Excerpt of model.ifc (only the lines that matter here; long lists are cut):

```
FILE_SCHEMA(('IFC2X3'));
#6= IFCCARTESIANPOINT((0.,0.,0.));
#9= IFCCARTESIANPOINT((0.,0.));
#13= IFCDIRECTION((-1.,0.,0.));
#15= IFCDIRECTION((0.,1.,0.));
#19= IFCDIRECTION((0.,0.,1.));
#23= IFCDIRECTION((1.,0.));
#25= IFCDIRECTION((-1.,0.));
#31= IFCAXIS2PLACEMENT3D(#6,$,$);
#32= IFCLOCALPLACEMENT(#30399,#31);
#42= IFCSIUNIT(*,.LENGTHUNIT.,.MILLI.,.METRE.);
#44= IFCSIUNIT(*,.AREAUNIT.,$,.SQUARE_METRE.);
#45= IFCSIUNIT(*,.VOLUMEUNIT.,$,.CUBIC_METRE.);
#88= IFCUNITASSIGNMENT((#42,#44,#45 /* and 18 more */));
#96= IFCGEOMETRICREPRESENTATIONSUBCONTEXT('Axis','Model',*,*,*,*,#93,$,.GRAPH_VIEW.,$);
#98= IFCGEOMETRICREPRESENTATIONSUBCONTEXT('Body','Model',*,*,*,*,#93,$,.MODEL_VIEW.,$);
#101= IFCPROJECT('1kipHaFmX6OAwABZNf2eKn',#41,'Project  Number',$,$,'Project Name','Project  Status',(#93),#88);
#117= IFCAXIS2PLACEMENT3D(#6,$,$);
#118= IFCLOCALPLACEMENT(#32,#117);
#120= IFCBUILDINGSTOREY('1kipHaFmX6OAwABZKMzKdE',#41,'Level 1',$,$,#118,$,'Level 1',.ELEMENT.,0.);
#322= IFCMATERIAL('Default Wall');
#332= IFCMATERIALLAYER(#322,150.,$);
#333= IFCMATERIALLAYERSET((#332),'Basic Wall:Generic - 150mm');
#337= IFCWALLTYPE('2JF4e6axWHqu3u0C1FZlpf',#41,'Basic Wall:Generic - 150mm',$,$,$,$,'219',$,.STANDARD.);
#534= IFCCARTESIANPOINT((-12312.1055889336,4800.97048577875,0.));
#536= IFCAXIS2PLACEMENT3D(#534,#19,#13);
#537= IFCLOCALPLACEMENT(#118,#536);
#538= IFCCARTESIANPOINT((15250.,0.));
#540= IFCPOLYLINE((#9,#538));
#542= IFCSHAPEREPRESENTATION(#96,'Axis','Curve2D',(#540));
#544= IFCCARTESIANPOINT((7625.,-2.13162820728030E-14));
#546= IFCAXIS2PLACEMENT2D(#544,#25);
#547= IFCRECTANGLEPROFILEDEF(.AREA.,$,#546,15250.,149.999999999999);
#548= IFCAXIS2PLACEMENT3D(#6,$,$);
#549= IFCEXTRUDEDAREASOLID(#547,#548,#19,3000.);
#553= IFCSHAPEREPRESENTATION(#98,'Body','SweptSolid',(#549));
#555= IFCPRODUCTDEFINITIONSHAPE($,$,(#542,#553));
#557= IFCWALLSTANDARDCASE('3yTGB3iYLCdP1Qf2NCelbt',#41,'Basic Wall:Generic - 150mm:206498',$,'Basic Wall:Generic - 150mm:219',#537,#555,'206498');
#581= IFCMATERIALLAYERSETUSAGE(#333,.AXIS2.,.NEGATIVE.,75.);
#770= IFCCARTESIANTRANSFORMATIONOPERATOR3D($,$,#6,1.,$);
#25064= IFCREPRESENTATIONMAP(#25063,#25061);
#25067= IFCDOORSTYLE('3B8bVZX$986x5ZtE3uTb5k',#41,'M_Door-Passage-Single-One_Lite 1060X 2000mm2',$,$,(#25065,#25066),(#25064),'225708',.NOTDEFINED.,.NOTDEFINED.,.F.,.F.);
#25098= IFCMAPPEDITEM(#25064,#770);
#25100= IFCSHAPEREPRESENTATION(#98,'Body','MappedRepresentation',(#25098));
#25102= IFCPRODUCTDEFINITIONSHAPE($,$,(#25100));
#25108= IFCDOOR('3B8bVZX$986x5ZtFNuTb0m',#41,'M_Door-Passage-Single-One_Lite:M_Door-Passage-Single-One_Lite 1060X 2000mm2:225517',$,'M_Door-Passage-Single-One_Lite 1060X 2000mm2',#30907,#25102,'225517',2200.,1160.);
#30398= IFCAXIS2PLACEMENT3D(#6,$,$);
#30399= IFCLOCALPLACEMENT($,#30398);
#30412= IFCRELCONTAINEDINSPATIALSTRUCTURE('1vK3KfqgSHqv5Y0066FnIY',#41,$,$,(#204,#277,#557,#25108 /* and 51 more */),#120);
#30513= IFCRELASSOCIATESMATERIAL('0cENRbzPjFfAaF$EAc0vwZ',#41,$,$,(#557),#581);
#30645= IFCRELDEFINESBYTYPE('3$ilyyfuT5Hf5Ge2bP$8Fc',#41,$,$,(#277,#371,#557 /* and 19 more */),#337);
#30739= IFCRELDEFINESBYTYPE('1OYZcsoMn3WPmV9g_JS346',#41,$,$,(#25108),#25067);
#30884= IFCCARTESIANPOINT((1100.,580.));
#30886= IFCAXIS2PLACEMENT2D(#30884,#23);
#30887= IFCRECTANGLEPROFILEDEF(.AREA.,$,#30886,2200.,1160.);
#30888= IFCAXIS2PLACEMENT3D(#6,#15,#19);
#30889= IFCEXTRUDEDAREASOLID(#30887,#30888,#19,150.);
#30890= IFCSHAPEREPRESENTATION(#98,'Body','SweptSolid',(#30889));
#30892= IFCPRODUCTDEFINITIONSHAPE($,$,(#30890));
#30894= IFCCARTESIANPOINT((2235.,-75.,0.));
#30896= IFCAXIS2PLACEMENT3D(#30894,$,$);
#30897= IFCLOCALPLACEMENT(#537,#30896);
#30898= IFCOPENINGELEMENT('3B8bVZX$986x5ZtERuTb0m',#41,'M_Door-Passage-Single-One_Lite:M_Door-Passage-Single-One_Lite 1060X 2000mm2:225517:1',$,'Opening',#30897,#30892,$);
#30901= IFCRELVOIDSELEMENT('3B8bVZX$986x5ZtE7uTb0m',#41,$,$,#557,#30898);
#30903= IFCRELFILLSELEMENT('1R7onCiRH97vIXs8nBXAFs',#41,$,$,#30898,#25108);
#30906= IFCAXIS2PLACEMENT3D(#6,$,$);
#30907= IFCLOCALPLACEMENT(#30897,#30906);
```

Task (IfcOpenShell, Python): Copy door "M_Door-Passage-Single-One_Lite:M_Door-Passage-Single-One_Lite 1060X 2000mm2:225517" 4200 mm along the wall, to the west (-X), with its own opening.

```python
import ifcopenshell
import ifcopenshell.api.feature
import ifcopenshell.api.geometry
import ifcopenshell.api.root
import ifcopenshell.geom
import ifcopenshell.util.element
import ifcopenshell.util.placement
import ifcopenshell.util.shape
import ifcopenshell.util.unit

model = ifcopenshell.open("model.ifc")
unit_scale = ifcopenshell.util.unit.calculate_unit_scale(model)
settings = ifcopenshell.geom.settings()


def volume(element):
    """Net volume in cubic metres, openings subtracted."""
    shape = ifcopenshell.geom.create_shape(settings, element)
    return ifcopenshell.util.shape.get_volume(shape.geometry)


def reuse_history(source, copy):
    """copy_class also copies each property set's owner history, people and application; keep the originals."""
    for rel in copy.IsDefinedBy:
        if rel.is_a("IfcRelDefinesByProperties") and (history := rel.RelatingPropertyDefinition.OwnerHistory):
            rel.RelatingPropertyDefinition.OwnerHistory = source.OwnerHistory
            ifcopenshell.util.element.remove_deep2(model, history)


door = model.by_guid("3B8bVZX$986x5ZtFNuTb0m")
opening = door.FillsVoids[0].RelatingOpeningElement
wall = opening.VoidsElements[0].RelatingBuildingElement
before = volume(wall)
shift = ifcopenshell.util.placement.get_local_placement(wall.ObjectPlacement)[:3, 0] * 4.2 / unit_scale

# copy_class copies the void relationship, type, container and properties, but no geometry.
new_opening = ifcopenshell.api.root.copy_class(model, product=opening)
new_opening.Representation = ifcopenshell.util.element.copy_deep(
    model, opening.Representation, exclude=["IfcGeometricRepresentationContext", "IfcRepresentationMap"]
)
new_opening.Name = "M_Door-Passage-Single-One_Lite:M_Door-Passage-Single-One_Lite 1060X 2000mm2"
new_door = ifcopenshell.api.root.copy_class(model, product=door)
new_door.Representation = ifcopenshell.util.element.copy_deep(
    model, door.Representation, exclude=["IfcGeometricRepresentationContext", "IfcRepresentationMap"]
)
new_door.Name = "M_Door-Passage-Single-One_Lite:M_Door-Passage-Single-One_Lite 1060X 2000mm2"
new_door.Tag = None
reuse_history(door, new_door)
fills = ifcopenshell.api.feature.add_filling(model, opening=new_opening, element=new_door)
fills.OwnerHistory = new_door.OwnerHistory  # required in IFC2X3

for old, new in ((opening, new_opening), (door, new_door)):
    matrix = ifcopenshell.util.placement.get_local_placement(old.ObjectPlacement)
    matrix[:3, 3] += shift
    ifcopenshell.api.geometry.edit_object_placement(model, product=new, matrix=matrix, is_si=False)

after = volume(wall)

print(f"wall volume {before:.3f} -> {after:.3f} m3")

model.write("model_updated.ifc")
```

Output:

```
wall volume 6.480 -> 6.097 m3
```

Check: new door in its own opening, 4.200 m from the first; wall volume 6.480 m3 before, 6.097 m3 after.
